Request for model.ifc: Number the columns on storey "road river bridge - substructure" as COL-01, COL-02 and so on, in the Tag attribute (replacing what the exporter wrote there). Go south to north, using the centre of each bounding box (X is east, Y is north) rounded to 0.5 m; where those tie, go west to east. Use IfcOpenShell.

First a look at what the model holds.

```python
import ifcopenshell
import ifcopenshell.util.element
import ifcopenshell.util.placement

model = ifcopenshell.open("model.ifc")
print(model.schema)
storey = next(s for s in model.by_type("IfcBuildingStorey") if s.Name == "road river bridge - substructure")
columns = [e for e in ifcopenshell.util.element.get_decomposition(storey) if e.is_a("IfcColumn")]
for e in sorted(columns, key=lambda e: e.id()):
    origin = ifcopenshell.util.placement.get_local_placement(e.ObjectPlacement)[:3, 3]
    print(e.id(), e.Tag, e.Name, origin.round(2) + 0.0, sep=" | ")
```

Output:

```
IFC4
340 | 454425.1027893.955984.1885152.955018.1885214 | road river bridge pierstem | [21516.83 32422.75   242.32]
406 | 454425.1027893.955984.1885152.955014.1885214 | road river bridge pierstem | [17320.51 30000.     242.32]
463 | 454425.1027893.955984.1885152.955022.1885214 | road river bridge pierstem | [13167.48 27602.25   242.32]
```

```python
import ifcopenshell
import ifcopenshell.geom
import ifcopenshell.util.element
import ifcopenshell.util.shape

model = ifcopenshell.open("model.ifc")
settings = ifcopenshell.geom.settings()
settings.set("use-world-coords", True)


def centre(element):
    shape = ifcopenshell.geom.create_shape(settings, element)
    return ifcopenshell.util.shape.get_bbox_centroid(shape.geometry)


storey = next(s for s in model.by_type("IfcBuildingStorey") if s.Name == "road river bridge - substructure")
columns = [e for e in ifcopenshell.util.element.get_decomposition(storey) if e.is_a("IfcColumn")]

# Insertion points can sit at a corner or the storey origin, so sort by the geometry (in metres).
centres = {e: centre(e) for e in columns}
columns.sort(key=lambda e: (round(centres[e][1] / 0.5), centres[e][0]))

for i, e in enumerate(columns, start=1):
    number = f"COL-{i:02d}"
    e.Tag = number
    print(e.id(), number)

model.write("model_v2.ifc")
```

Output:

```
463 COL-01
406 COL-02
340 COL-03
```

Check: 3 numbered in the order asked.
